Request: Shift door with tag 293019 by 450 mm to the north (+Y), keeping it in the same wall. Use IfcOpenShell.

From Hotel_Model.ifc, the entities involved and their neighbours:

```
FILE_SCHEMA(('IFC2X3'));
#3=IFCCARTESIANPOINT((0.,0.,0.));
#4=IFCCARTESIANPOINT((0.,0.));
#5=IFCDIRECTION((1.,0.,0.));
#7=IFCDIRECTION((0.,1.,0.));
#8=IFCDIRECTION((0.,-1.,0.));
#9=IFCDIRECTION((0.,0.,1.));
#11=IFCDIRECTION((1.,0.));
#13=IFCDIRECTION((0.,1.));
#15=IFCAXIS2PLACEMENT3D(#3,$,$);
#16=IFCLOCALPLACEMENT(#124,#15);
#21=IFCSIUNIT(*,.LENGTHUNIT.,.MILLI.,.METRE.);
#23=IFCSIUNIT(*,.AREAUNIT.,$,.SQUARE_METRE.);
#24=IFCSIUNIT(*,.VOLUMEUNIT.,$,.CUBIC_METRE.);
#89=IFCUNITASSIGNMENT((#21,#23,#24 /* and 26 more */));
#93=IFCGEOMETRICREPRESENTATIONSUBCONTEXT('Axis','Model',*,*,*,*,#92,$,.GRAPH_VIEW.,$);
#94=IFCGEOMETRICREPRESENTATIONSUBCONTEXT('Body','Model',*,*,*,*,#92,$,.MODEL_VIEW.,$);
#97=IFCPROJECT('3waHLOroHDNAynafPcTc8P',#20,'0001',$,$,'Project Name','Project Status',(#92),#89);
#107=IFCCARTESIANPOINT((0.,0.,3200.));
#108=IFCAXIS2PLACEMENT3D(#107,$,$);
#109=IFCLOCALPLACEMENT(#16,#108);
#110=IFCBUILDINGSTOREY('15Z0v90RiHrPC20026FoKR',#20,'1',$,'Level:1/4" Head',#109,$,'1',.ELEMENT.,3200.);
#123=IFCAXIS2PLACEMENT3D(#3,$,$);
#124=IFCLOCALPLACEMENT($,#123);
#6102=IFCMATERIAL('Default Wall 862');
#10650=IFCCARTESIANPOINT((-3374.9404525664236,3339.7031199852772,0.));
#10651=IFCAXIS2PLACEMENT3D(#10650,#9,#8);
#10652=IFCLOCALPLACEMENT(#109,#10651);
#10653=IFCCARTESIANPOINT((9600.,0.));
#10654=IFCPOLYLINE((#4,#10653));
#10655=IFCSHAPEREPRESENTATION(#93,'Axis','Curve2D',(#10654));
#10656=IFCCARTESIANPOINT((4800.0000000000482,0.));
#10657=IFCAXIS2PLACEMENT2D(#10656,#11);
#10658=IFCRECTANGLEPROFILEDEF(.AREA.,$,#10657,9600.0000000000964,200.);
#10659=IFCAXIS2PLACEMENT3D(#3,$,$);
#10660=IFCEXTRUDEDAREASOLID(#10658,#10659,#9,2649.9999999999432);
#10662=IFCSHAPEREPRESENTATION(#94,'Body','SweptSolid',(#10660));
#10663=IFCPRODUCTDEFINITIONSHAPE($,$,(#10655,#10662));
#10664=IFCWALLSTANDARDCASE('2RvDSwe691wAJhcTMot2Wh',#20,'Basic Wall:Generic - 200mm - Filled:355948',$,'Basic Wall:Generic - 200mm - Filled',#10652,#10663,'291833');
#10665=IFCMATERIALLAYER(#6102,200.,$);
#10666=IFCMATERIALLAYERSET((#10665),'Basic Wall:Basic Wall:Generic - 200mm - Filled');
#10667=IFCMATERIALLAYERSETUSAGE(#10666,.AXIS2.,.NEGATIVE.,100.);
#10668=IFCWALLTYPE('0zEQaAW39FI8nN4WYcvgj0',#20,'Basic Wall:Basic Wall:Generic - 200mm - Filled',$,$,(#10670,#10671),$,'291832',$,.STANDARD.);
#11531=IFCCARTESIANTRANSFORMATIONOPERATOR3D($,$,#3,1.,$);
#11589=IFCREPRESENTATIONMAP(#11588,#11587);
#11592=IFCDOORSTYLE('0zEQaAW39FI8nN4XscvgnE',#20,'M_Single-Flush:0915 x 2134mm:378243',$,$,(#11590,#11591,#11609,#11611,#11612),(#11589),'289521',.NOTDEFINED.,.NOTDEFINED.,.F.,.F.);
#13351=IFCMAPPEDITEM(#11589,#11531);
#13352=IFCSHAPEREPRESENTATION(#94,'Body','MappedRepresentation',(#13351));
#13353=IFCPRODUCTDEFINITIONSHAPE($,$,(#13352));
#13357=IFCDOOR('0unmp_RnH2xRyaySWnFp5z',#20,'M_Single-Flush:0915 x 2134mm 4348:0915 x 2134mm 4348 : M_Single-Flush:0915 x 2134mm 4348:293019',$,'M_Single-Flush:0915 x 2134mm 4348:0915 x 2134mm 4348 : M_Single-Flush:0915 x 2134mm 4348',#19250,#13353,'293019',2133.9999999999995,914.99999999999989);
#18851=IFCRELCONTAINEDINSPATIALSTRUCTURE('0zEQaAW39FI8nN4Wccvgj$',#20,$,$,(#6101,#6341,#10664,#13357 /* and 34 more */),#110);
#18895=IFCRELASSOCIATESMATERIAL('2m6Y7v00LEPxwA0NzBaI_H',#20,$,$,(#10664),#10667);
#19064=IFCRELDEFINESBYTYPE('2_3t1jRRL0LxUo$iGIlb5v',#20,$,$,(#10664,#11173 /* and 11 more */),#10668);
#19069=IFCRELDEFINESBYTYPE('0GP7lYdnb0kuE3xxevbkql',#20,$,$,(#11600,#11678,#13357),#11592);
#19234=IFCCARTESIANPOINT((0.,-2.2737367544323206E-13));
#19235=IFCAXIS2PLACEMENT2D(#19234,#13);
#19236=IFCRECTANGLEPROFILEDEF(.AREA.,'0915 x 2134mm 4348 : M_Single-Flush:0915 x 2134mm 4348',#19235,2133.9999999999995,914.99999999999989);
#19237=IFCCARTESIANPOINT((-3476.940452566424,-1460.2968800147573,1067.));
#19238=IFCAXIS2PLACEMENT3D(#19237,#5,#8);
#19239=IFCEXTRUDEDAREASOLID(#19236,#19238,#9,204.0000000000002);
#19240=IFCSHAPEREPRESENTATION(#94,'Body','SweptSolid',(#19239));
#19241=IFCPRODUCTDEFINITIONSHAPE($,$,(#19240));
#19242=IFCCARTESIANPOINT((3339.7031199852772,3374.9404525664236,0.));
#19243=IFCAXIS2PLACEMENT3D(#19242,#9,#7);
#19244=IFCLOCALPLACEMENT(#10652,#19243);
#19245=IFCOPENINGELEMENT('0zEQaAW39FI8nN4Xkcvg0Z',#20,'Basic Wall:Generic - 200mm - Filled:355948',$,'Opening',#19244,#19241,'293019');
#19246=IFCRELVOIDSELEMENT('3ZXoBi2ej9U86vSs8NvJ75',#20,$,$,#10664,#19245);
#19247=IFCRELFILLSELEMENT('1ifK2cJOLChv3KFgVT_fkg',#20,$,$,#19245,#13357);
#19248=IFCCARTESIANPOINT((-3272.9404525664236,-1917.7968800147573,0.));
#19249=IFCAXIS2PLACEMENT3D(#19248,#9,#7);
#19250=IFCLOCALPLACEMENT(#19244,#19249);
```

```python
import ifcopenshell
import ifcopenshell.api.geometry
import ifcopenshell.util.placement
import ifcopenshell.util.unit

model = ifcopenshell.open("Hotel_Model.ifc")
unit_scale = ifcopenshell.util.unit.calculate_unit_scale(model)

door = model.by_guid("0unmp_RnH2xRyaySWnFp5z")
opening = door.FillsVoids[0].RelatingOpeningElement
wall = opening.VoidsElements[0].RelatingBuildingElement

wall_matrix = ifcopenshell.util.placement.get_local_placement(wall.ObjectPlacement)
shift = wall_matrix[:3, 0] * -0.45 / unit_scale
before = ifcopenshell.util.placement.get_local_placement(door.ObjectPlacement)[:3, 3].copy()

# The door is placed relative to its opening, so it follows when the opening moves.
matrix = ifcopenshell.util.placement.get_local_placement(opening.ObjectPlacement)
matrix[:3, 3] += shift
ifcopenshell.api.geometry.edit_object_placement(
    model, product=opening, matrix=matrix, is_si=False, should_transform_children=True
)

after = ifcopenshell.util.placement.get_local_placement(door.ObjectPlacement)[:3, 3]
print("door moved by", (after - before).round(3) + 0.0)

model.write("Hotel_Model_edited.ifc")
```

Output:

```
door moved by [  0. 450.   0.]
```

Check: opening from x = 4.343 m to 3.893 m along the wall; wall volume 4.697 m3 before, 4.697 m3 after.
